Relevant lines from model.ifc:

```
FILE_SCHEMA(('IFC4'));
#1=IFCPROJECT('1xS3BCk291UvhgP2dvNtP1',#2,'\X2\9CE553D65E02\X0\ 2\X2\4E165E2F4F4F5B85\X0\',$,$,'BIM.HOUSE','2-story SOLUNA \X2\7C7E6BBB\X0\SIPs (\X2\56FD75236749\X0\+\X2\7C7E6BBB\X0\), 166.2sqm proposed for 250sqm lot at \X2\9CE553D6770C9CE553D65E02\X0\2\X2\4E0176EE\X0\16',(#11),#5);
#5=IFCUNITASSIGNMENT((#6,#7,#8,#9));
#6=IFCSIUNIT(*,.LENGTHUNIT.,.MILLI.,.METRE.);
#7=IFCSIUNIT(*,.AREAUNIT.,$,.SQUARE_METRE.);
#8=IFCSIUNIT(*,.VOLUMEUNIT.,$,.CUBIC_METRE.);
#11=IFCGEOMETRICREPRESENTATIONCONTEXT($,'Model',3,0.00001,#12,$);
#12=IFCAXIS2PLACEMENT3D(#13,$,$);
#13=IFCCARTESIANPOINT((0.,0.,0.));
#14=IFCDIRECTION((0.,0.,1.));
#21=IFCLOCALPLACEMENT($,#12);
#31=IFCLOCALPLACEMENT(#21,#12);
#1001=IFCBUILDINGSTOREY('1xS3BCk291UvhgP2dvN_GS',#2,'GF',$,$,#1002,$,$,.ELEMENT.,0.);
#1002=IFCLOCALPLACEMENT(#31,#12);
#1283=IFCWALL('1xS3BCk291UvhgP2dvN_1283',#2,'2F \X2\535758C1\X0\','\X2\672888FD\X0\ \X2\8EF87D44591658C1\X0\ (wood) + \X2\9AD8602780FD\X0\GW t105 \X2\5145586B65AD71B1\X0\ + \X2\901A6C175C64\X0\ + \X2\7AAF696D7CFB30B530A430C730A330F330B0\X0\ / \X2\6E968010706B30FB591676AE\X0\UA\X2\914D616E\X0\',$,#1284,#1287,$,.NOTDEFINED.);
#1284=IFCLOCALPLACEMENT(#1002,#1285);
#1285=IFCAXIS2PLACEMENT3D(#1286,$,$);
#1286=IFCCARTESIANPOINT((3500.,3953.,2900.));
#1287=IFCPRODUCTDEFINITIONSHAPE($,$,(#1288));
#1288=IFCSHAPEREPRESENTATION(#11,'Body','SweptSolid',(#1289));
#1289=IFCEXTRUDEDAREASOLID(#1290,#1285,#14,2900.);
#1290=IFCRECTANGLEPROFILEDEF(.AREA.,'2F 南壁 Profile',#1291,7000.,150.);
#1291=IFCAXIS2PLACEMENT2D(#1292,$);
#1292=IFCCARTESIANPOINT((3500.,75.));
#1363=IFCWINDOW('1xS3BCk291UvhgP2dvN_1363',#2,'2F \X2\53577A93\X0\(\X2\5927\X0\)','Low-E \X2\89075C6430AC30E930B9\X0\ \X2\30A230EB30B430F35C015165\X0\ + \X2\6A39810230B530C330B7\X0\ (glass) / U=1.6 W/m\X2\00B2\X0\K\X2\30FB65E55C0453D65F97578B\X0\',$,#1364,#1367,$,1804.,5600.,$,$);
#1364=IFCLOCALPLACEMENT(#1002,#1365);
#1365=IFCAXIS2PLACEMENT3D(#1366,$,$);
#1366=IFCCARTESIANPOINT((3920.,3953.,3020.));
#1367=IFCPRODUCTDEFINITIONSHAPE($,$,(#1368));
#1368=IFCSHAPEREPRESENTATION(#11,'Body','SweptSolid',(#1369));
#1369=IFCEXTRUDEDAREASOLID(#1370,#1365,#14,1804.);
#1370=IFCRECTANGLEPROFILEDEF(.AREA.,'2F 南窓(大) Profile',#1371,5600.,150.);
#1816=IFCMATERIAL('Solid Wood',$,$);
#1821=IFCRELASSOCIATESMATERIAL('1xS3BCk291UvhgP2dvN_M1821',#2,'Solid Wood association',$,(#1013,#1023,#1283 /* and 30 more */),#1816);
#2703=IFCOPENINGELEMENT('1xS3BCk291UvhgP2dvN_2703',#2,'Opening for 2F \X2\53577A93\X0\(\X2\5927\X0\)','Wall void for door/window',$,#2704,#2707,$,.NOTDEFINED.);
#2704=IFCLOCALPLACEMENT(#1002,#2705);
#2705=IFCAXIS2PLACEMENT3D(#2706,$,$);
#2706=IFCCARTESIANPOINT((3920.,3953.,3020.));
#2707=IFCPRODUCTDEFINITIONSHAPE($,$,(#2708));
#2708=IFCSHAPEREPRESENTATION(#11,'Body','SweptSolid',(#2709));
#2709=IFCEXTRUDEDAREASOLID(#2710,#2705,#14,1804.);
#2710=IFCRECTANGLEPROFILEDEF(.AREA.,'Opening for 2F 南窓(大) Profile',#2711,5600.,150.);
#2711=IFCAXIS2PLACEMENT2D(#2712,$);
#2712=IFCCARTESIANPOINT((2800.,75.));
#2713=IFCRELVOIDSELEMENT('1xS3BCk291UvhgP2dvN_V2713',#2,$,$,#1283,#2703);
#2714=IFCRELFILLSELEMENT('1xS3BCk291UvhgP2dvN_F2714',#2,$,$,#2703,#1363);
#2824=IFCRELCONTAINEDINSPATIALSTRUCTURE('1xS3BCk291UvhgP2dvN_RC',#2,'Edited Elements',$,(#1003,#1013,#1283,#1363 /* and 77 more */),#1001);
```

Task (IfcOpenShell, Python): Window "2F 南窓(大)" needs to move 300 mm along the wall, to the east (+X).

```python
import ifcopenshell
import ifcopenshell.api.geometry
import ifcopenshell.util.placement
import ifcopenshell.util.unit

model = ifcopenshell.open("model.ifc")
unit_scale = ifcopenshell.util.unit.calculate_unit_scale(model)

window = model.by_guid("1xS3BCk291UvhgP2dvN_1363")
opening = window.FillsVoids[0].RelatingOpeningElement
wall = opening.VoidsElements[0].RelatingBuildingElement

wall_matrix = ifcopenshell.util.placement.get_local_placement(wall.ObjectPlacement)
shift = wall_matrix[:3, 0] * 0.3 / unit_scale
before = ifcopenshell.util.placement.get_local_placement(window.ObjectPlacement)[:3, 3].copy()

# The window is not placed relative to its opening, so move both.
for product in (opening, window):
    matrix = ifcopenshell.util.placement.get_local_placement(product.ObjectPlacement)
    matrix[:3, 3] += shift
    ifcopenshell.api.geometry.edit_object_placement(model, product=product, matrix=matrix, is_si=False)

after = ifcopenshell.util.placement.get_local_placement(window.ObjectPlacement)[:3, 3]
print("window moved by", (after - before).round(3) + 0.0)

model.write("model_v2.ifc")
```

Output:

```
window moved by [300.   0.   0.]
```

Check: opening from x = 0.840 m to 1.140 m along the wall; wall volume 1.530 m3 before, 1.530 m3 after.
